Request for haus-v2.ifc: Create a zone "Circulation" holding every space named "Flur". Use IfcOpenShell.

First a look at what the model holds.

```python
import ifcopenshell

model = ifcopenshell.open("haus-v2.ifc")
print(model.schema)
seen = {}
for space in model.by_type("IfcSpace"):
    seen[space.LongName] = seen.get(space.LongName, 0) + 1
for name, count in sorted(seen.items(), key=str):
    print(count, "x", name)
print("zones:", [z.Name for z in model.by_type("IfcZone")][:20])
```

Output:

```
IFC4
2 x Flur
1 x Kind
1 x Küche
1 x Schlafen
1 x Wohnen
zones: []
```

```python
import ifcopenshell
import ifcopenshell.api.group
import ifcopenshell.api.root

model = ifcopenshell.open("haus-v2.ifc")

names = {"Flur"}
spaces = [s for s in model.by_type("IfcSpace") if s.LongName in names]

zone = ifcopenshell.api.root.create_entity(model, ifc_class="IfcZone", name="Circulation")
ifcopenshell.api.group.assign_group(model, products=spaces, group=zone)
print(len(spaces), "spaces in", zone.Name)

model.write("haus-v2_rev.ifc")
```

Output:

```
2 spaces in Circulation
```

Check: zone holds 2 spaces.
